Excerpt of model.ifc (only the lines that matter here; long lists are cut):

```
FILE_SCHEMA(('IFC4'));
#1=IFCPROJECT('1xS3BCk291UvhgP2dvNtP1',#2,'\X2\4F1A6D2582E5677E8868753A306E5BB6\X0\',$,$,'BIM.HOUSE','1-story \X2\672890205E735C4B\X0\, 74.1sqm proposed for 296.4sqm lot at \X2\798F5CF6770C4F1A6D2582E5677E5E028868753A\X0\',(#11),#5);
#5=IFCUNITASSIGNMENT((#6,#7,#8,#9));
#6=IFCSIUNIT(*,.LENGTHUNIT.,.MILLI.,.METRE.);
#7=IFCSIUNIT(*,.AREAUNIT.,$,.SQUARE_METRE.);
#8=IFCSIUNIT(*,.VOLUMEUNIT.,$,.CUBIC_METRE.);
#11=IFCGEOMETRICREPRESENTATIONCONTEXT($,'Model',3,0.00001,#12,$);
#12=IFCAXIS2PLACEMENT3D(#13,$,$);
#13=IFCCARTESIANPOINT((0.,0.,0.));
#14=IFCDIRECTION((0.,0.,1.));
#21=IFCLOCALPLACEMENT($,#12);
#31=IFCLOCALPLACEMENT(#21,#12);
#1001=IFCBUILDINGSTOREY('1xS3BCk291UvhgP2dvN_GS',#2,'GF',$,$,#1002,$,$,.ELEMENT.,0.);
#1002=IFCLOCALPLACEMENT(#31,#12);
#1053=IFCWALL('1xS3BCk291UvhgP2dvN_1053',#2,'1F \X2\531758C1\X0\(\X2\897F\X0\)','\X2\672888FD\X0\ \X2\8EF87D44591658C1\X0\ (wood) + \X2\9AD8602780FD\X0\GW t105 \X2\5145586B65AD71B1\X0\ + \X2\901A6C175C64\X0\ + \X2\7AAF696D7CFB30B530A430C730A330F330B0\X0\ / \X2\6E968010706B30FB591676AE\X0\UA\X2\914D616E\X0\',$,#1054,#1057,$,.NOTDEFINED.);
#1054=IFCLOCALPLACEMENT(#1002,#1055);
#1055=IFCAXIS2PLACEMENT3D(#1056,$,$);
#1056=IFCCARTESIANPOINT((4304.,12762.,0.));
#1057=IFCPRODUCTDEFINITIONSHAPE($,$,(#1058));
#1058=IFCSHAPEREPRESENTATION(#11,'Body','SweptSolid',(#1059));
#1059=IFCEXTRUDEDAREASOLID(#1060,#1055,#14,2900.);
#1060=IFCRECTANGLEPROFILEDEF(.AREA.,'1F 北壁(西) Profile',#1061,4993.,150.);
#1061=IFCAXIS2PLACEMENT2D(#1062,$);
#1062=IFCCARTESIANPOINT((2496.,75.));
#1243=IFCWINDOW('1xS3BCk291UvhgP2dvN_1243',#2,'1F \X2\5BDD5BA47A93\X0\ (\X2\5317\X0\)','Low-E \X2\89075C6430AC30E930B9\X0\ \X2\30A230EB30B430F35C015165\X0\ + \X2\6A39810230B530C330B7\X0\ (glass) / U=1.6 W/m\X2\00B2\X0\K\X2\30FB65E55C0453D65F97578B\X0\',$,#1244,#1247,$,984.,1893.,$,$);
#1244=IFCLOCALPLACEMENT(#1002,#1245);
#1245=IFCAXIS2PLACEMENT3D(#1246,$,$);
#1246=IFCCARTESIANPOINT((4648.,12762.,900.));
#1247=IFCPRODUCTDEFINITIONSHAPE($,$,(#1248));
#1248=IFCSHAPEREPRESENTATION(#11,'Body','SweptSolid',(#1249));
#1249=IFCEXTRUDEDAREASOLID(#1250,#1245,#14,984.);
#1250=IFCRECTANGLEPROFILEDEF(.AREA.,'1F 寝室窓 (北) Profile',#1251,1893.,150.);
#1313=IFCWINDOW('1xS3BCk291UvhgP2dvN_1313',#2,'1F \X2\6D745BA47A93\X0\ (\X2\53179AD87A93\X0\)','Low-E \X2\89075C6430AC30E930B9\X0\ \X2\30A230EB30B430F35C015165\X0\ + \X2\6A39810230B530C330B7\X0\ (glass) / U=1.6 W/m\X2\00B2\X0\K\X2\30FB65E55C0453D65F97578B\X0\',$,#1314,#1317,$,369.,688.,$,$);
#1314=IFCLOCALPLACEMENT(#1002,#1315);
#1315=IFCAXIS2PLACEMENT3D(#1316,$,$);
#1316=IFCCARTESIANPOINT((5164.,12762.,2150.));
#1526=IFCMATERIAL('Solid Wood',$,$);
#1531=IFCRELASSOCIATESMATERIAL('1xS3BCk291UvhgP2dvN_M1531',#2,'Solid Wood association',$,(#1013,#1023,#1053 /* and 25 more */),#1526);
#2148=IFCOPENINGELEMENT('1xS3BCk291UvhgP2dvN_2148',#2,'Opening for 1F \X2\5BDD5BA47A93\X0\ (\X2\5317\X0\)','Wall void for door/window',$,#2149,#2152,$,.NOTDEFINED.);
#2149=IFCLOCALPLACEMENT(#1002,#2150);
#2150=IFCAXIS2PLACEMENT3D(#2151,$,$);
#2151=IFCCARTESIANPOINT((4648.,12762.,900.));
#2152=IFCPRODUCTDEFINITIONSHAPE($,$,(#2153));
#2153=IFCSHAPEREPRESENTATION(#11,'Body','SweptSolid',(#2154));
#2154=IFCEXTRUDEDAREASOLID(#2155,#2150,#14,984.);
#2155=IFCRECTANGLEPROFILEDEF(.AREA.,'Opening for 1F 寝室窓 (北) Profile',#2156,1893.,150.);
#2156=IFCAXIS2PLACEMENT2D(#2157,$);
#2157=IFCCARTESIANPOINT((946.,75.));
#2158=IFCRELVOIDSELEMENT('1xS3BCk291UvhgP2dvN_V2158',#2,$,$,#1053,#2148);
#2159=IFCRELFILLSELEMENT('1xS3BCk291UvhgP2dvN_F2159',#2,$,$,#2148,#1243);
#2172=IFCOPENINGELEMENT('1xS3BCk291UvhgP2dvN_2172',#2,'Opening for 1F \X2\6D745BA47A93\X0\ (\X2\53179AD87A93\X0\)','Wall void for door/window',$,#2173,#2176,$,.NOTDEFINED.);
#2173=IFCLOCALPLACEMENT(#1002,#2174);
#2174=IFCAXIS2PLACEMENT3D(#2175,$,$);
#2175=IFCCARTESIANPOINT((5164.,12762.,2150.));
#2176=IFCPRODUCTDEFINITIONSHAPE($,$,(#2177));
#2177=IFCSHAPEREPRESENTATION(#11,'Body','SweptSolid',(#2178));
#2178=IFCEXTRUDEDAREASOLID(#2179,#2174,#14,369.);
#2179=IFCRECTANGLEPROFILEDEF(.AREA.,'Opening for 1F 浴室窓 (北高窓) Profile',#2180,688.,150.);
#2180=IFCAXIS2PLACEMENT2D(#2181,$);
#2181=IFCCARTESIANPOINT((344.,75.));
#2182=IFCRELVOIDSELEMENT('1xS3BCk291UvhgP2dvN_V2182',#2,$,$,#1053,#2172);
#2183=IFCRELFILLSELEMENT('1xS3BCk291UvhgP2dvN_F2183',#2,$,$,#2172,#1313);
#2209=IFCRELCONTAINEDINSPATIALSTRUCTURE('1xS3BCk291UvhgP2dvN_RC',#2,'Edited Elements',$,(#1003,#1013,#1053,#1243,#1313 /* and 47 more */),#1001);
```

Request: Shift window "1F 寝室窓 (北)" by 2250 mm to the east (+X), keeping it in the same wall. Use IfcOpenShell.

```python
import ifcopenshell
import ifcopenshell.api.geometry
import ifcopenshell.util.placement
import ifcopenshell.util.unit

model = ifcopenshell.open("model.ifc")
unit_scale = ifcopenshell.util.unit.calculate_unit_scale(model)

window = model.by_guid("1xS3BCk291UvhgP2dvN_1243")
opening = window.FillsVoids[0].RelatingOpeningElement
wall = opening.VoidsElements[0].RelatingBuildingElement

wall_matrix = ifcopenshell.util.placement.get_local_placement(wall.ObjectPlacement)
shift = wall_matrix[:3, 0] * 2.25 / unit_scale
before = ifcopenshell.util.placement.get_local_placement(window.ObjectPlacement)[:3, 3].copy()

# The window is not placed relative to its opening, so move both.
for product in (opening, window):
    matrix = ifcopenshell.util.placement.get_local_placement(product.ObjectPlacement)
    matrix[:3, 3] += shift
    ifcopenshell.api.geometry.edit_object_placement(model, product=product, matrix=matrix, is_si=False)

after = ifcopenshell.util.placement.get_local_placement(window.ObjectPlacement)[:3, 3]
print("window moved by", (after - before).round(3) + 0.0)

model.write("model-out.ifc")
```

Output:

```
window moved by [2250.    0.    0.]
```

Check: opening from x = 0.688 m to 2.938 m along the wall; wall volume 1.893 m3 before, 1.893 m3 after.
